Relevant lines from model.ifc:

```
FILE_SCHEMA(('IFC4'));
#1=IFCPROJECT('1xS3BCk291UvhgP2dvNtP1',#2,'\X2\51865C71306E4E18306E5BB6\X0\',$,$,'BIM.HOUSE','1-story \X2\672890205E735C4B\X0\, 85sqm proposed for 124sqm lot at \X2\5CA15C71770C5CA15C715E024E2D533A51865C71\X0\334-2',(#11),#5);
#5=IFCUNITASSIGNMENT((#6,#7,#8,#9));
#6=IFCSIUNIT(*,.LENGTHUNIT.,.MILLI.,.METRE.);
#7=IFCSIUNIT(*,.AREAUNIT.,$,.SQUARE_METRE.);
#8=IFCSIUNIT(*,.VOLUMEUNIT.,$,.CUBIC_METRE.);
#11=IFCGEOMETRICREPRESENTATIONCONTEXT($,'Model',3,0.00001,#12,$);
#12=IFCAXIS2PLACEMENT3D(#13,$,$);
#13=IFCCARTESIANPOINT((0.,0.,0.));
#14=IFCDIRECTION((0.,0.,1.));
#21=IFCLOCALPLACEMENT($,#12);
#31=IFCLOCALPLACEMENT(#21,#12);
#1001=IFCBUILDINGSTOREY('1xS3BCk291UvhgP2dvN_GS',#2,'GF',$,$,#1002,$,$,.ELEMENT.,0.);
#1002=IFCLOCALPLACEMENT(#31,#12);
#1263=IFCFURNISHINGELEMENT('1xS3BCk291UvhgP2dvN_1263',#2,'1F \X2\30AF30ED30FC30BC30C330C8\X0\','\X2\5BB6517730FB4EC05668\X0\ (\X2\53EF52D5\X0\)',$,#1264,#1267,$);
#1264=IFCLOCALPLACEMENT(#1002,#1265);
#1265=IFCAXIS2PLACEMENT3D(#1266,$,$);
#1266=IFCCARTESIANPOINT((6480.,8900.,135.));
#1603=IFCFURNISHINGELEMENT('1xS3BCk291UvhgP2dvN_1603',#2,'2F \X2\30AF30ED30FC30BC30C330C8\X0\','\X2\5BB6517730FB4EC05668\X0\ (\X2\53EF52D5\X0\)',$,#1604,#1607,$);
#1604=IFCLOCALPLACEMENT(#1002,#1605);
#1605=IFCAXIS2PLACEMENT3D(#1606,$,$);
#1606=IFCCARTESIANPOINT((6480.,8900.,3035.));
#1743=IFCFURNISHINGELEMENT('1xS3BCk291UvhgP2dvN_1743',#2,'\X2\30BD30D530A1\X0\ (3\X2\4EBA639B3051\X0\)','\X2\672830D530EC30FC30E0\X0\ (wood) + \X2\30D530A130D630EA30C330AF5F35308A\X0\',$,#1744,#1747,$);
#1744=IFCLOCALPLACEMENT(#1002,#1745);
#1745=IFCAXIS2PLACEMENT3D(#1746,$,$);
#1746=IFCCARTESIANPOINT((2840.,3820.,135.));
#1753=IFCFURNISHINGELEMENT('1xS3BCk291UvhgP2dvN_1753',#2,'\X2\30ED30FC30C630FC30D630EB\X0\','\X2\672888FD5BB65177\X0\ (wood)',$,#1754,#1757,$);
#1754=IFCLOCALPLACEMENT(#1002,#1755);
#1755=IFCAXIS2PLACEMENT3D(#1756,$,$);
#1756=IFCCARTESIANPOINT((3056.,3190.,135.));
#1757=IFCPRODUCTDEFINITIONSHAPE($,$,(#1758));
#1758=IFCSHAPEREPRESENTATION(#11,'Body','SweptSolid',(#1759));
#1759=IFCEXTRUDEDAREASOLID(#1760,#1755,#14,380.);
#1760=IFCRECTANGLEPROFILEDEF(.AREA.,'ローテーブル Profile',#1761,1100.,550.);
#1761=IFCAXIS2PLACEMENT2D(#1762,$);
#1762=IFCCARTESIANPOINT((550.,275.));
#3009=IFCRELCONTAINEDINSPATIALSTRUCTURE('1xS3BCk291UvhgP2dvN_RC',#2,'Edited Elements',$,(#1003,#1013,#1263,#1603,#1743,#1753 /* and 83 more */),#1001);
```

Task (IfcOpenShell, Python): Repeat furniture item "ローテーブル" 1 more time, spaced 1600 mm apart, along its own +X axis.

```python
import ifcopenshell
import ifcopenshell.api.geometry
import ifcopenshell.api.root
import ifcopenshell.util.element
import ifcopenshell.util.placement
import ifcopenshell.util.unit

model = ifcopenshell.open("model.ifc")
unit_scale = ifcopenshell.util.unit.calculate_unit_scale(model)


def reuse_history(source, copy):
    """copy_class also copies each property set's owner history, people and application; keep the originals."""
    for rel in copy.IsDefinedBy:
        if rel.is_a("IfcRelDefinesByProperties") and (history := rel.RelatingPropertyDefinition.OwnerHistory):
            rel.RelatingPropertyDefinition.OwnerHistory = source.OwnerHistory
            ifcopenshell.util.element.remove_deep2(model, history)


source = model.by_guid("1xS3BCk291UvhgP2dvN_1753")
base = ifcopenshell.util.placement.get_local_placement(source.ObjectPlacement)
step = base[:3, 0] * 1.6 / unit_scale

for i in range(1, 2):
    copy = ifcopenshell.api.root.copy_class(model, product=source)
    copy.Representation = ifcopenshell.util.element.copy_deep(
        model, source.Representation, exclude=["IfcGeometricRepresentationContext", "IfcRepresentationMap"]
    )
    reuse_history(source, copy)
    matrix = base.copy()
    matrix[:3, 3] += i * step
    print("added at", matrix[:3, 3].round(3) + 0.0)
    ifcopenshell.api.geometry.edit_object_placement(model, product=copy, matrix=matrix, is_si=False)

model.write("model_v2.ifc")
```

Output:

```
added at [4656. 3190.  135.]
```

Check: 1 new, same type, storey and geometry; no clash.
